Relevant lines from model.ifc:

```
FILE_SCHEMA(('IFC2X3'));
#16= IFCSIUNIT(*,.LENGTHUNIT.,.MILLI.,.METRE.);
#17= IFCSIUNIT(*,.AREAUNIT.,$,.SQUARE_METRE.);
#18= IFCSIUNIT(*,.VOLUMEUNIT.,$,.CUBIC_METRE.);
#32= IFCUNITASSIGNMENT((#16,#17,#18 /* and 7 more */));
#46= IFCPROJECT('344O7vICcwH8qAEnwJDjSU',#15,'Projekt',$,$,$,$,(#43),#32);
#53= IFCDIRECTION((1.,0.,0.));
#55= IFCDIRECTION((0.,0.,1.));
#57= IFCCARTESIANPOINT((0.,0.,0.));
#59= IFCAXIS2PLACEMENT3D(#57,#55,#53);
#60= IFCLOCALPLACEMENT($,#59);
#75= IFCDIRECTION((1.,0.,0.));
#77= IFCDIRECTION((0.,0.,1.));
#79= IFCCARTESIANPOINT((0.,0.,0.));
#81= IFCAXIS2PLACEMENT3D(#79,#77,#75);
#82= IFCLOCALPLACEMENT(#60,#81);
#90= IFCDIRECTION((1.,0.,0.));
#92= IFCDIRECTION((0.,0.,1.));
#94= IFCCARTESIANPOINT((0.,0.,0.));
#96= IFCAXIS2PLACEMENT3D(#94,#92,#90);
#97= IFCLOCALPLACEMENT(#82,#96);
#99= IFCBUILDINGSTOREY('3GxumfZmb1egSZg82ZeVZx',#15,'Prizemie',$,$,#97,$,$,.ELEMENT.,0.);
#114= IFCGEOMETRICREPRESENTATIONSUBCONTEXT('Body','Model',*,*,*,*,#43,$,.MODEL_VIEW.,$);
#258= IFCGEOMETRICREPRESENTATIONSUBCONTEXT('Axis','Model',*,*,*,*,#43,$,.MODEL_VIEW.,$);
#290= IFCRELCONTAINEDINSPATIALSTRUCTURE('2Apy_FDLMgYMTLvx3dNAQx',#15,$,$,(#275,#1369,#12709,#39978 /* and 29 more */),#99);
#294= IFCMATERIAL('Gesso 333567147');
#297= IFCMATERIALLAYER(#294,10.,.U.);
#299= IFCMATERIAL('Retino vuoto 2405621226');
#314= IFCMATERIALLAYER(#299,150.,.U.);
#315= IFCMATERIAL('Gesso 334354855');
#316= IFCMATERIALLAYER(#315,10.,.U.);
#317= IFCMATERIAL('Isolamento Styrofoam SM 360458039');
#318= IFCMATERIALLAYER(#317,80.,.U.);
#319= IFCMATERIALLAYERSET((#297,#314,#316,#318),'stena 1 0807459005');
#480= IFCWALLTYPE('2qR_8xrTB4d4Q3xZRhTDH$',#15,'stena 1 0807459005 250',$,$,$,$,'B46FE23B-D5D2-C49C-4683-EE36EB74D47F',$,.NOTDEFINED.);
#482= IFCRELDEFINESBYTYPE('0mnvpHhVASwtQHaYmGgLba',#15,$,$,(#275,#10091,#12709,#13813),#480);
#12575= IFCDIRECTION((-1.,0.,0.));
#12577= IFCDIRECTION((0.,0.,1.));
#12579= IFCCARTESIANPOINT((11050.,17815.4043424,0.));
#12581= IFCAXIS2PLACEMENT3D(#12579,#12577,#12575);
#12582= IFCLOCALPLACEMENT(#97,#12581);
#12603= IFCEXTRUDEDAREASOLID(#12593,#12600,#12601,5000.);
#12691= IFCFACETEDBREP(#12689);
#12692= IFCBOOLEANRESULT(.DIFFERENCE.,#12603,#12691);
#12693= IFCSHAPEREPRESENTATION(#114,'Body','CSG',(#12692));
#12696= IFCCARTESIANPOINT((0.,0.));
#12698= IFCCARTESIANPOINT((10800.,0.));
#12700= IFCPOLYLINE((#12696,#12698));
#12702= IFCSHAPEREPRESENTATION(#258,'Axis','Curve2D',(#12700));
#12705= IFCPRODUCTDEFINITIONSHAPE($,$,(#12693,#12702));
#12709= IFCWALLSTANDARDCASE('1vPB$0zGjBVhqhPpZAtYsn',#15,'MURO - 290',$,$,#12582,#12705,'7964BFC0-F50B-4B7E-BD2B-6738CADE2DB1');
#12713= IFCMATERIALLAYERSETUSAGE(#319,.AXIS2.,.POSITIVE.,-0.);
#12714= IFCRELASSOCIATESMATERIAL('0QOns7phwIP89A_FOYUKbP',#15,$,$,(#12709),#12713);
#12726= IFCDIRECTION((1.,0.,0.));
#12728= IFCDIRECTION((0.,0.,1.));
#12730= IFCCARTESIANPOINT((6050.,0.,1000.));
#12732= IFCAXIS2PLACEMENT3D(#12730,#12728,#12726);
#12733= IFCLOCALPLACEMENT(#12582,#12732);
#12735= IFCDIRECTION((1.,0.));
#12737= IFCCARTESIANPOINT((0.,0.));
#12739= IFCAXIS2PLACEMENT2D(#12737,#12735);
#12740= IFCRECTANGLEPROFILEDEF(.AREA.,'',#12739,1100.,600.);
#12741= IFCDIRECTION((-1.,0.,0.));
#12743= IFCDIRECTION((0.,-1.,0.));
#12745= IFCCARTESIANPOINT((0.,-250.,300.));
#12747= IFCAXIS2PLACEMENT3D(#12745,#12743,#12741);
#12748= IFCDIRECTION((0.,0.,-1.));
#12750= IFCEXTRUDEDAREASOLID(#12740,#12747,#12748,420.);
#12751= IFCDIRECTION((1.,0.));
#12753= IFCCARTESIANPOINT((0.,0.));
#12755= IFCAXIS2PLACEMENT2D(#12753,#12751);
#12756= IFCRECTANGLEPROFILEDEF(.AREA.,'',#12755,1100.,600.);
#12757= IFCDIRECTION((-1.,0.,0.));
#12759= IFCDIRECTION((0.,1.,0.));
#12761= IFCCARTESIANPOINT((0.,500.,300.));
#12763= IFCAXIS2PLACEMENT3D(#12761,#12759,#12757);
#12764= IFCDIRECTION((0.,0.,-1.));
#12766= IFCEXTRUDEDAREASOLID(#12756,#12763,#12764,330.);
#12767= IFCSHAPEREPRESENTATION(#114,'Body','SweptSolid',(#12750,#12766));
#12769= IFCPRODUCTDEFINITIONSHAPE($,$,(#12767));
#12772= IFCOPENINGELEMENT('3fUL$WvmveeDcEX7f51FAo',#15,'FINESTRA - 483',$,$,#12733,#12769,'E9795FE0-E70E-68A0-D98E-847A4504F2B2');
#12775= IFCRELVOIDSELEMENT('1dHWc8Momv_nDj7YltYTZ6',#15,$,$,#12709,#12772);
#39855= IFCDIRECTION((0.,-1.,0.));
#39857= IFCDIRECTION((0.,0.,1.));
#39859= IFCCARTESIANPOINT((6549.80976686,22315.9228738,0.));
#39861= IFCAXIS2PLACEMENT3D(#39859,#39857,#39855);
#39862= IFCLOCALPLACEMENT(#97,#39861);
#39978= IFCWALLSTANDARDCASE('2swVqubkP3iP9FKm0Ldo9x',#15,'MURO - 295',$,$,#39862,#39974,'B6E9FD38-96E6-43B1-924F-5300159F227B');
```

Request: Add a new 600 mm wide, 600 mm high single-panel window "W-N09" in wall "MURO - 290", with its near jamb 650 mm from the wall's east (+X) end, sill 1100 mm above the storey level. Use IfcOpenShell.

```python
import numpy as np
import ifcopenshell
import ifcopenshell.api.feature
import ifcopenshell.api.geometry
import ifcopenshell.api.root
import ifcopenshell.api.spatial
import ifcopenshell.api.type
import ifcopenshell.geom
import ifcopenshell.util.element
import ifcopenshell.util.placement
import ifcopenshell.util.representation
import ifcopenshell.util.shape
import ifcopenshell.util.unit

model = ifcopenshell.open("model.ifc")
unit_scale = ifcopenshell.util.unit.calculate_unit_scale(model)
settings = ifcopenshell.geom.settings()


def volume(element):
    """Net volume in cubic metres, openings subtracted."""
    shape = ifcopenshell.geom.create_shape(settings, element)
    return ifcopenshell.util.shape.get_volume(shape.geometry)


wall = model.by_guid("1vPB$0zGjBVhqhPpZAtYsn")
storey = ifcopenshell.util.element.get_container(wall, ifc_class="IfcBuildingStorey")
context = ifcopenshell.util.representation.get_context(model, "Model", "Body", "MODEL_VIEW")
before = volume(wall)

width, height, from_end, sill = 0.6, 0.6, 0.65, 1.1  # metres

# The wall runs along its own X axis, and the end named is its -X end.
wall_shape = ifcopenshell.geom.create_shape(settings, wall)
x, y, z = ifcopenshell.util.shape.get_vertices(wall_shape.geometry).T
start = x.min() + from_end
face, thickness = float(y.min()), float(y.max() - y.min())
wall_matrix = ifcopenshell.util.placement.get_local_placement(wall.ObjectPlacement)
level = ifcopenshell.util.placement.get_local_placement(storey.ObjectPlacement)[2, 3]


def in_wall(x, y):
    """Placement at x, y metres in the wall's axes, at sill height."""
    matrix = wall_matrix.copy()
    matrix[:, 3] = wall_matrix @ np.array([x / unit_scale, y / unit_scale, 0.0, 1.0])
    matrix[2, 3] = level + sill / unit_scale
    return matrix


# Opening: a box that overshoots both wall faces by 50 mm.
opening = ifcopenshell.api.root.create_entity(model, ifc_class="IfcOpeningElement")
box = ifcopenshell.api.geometry.add_wall_representation(
    model, context=context, length=width, height=height, thickness=thickness + 0.1
)
ifcopenshell.api.geometry.assign_representation(model, product=opening, representation=box)
ifcopenshell.api.geometry.edit_object_placement(model, product=opening, matrix=in_wall(start, face - 0.05), is_si=False)
ifcopenshell.api.feature.add_feature(model, feature=opening, element=wall)

window = ifcopenshell.api.root.create_entity(model, ifc_class="IfcWindow", name="W-N09")
window.OverallWidth, window.OverallHeight = width / unit_scale, height / unit_scale
body = ifcopenshell.api.geometry.add_window_representation(
    model,
    context=context,
    overall_width=window.OverallWidth,
    overall_height=window.OverallHeight,
    partition_type="SINGLE_PANEL",
)
ifcopenshell.api.geometry.assign_representation(model, product=window, representation=body)
ifcopenshell.api.spatial.assign_container(model, products=[window], relating_structure=storey)
fills = ifcopenshell.api.feature.add_filling(model, opening=opening, element=window)
fills.OwnerHistory = window.OwnerHistory  # required in IFC2X3

# IFC2X3 keeps the operation on the window style.
style = ifcopenshell.api.root.create_entity(model, ifc_class="IfcWindowStyle", name="W-N09")
style.OperationType, style.ConstructionType = "SINGLE_PANEL", "NOTDEFINED"
style.ParameterTakesPrecedence = style.Sizeable = False
ifcopenshell.api.type.assign_type(model, related_objects=[window], relating_type=style)

# Centre the window in the wall's thickness.
ifcopenshell.api.geometry.edit_object_placement(model, product=window, matrix=in_wall(start, face), is_si=False)
window_shape = ifcopenshell.geom.create_shape(settings, window)
depth = ifcopenshell.util.shape.get_vertices(window_shape.geometry)[:, 1]
offset = face + thickness / 2 - (depth.min() + depth.max()) / 2
ifcopenshell.api.geometry.edit_object_placement(model, product=window, matrix=in_wall(start, offset), is_si=False)

after = volume(wall)

print(f"wall volume {before:.3f} -> {after:.3f} m3")

model.write("model-out.ifc")
```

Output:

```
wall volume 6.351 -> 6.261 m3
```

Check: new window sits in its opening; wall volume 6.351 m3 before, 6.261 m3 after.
